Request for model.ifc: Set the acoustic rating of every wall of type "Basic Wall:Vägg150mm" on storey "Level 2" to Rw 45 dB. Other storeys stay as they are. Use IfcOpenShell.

First a look at what the model holds.

```python
import ifcopenshell
import ifcopenshell.util.element

model = ifcopenshell.open("model.ifc")
print(model.schema)
storey = next(s for s in model.by_type("IfcBuildingStorey") if s.Name == "Level 2")
walls = [e for e in ifcopenshell.util.element.get_decomposition(storey) if e.is_a("IfcWall")]
seen = {}
for e in walls:
    element_type = ifcopenshell.util.element.get_type(e)
    key = (element_type.Name if element_type != e and element_type else None, ifcopenshell.util.element.get_pset(e, "Pset_WallCommon", "AcousticRating"))
    seen[key] = seen.get(key, 0) + 1
for (name, value), count in sorted(seen.items(), key=str):
    print(count, "x", name, "|", value)
```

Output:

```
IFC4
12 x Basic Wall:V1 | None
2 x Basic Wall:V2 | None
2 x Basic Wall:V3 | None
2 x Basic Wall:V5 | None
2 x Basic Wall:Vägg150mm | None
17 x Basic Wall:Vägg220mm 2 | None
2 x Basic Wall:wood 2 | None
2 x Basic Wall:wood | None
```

```python
import ifcopenshell
import ifcopenshell.api.pset
import ifcopenshell.util.element

model = ifcopenshell.open("model.ifc")

storey = next(s for s in model.by_type("IfcBuildingStorey") if s.Name == "Level 2")
walls = [e for e in ifcopenshell.util.element.get_decomposition(storey) if e.is_a("IfcWall")]

count = 0
for e in walls:
    element_type = ifcopenshell.util.element.get_type(e)
    if element_type in (None, e) or element_type.Name != "Basic Wall:Vägg150mm":
        continue
    # add_pset returns the element's existing set when there is one.
    pset = ifcopenshell.api.pset.add_pset(model, product=e, name="Pset_WallCommon")
    ifcopenshell.api.pset.edit_pset(model, pset=pset, properties={"AcousticRating": "Rw 45 dB"})
    count += 1

print(count, "walls updated")

model.write("model_v2.ifc")
```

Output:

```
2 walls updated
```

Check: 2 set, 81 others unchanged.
